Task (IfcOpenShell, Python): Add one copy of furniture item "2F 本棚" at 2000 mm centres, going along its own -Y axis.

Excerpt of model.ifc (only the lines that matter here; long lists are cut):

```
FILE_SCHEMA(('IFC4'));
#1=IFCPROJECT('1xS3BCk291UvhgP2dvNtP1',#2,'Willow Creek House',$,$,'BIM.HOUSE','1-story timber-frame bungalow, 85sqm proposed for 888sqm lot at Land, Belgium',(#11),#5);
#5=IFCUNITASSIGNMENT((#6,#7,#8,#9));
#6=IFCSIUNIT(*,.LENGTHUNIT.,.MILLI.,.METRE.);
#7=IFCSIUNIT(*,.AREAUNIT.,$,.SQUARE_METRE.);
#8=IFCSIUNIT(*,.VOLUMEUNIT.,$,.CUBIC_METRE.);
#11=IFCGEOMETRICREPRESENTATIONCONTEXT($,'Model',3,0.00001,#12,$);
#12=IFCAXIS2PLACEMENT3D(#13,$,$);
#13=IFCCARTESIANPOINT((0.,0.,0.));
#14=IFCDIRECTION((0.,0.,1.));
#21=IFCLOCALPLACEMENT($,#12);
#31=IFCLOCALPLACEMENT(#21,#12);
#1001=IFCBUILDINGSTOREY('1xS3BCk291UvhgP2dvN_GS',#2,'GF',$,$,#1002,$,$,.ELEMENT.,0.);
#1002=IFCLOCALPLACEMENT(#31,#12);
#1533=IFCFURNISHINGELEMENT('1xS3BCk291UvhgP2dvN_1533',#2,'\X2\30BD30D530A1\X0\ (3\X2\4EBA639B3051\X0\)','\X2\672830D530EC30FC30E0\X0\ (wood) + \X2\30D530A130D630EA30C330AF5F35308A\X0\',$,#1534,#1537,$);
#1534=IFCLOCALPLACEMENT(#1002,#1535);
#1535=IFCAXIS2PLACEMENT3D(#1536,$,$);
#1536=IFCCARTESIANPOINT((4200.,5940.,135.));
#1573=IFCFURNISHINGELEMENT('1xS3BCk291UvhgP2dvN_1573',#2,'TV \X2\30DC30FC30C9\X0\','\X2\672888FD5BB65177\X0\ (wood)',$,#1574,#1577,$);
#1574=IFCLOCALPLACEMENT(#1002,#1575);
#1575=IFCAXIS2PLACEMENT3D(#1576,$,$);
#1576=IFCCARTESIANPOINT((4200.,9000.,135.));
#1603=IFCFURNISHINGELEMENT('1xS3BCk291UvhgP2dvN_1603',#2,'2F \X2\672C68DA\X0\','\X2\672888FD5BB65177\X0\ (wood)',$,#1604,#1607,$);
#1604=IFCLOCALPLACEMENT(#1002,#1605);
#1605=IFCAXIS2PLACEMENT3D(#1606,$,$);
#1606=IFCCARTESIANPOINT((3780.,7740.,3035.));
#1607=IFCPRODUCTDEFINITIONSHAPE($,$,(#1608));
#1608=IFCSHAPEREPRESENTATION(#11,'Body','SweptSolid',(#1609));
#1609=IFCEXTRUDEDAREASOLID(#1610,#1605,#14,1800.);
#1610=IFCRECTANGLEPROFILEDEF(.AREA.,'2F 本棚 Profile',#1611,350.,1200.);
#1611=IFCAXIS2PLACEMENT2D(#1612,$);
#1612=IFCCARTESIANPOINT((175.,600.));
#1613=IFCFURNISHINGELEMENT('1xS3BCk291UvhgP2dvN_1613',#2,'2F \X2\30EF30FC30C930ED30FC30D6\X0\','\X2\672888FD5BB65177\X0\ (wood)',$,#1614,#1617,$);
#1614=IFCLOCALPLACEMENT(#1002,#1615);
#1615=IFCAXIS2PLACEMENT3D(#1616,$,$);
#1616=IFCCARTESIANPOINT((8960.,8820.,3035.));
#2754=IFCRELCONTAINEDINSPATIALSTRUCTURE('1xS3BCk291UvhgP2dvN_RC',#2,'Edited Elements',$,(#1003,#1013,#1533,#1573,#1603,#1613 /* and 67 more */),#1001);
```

```python
import ifcopenshell
import ifcopenshell.api.geometry
import ifcopenshell.api.root
import ifcopenshell.util.element
import ifcopenshell.util.placement
import ifcopenshell.util.unit

model = ifcopenshell.open("model.ifc")
unit_scale = ifcopenshell.util.unit.calculate_unit_scale(model)


def reuse_history(source, copy):
    """copy_class also copies each property set's owner history, people and application; keep the originals."""
    for rel in copy.IsDefinedBy:
        if rel.is_a("IfcRelDefinesByProperties") and (history := rel.RelatingPropertyDefinition.OwnerHistory):
            rel.RelatingPropertyDefinition.OwnerHistory = source.OwnerHistory
            ifcopenshell.util.element.remove_deep2(model, history)


source = model.by_guid("1xS3BCk291UvhgP2dvN_1603")
base = ifcopenshell.util.placement.get_local_placement(source.ObjectPlacement)
step = -base[:3, 1] * 2 / unit_scale

for i in range(1, 2):
    copy = ifcopenshell.api.root.copy_class(model, product=source)
    copy.Representation = ifcopenshell.util.element.copy_deep(
        model, source.Representation, exclude=["IfcGeometricRepresentationContext", "IfcRepresentationMap"]
    )
    reuse_history(source, copy)
    matrix = base.copy()
    matrix[:3, 3] += i * step
    print("added at", matrix[:3, 3].round(3) + 0.0)
    ifcopenshell.api.geometry.edit_object_placement(model, product=copy, matrix=matrix, is_si=False)

model.write("model_v2.ifc")
```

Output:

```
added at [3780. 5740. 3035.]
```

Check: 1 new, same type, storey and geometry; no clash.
